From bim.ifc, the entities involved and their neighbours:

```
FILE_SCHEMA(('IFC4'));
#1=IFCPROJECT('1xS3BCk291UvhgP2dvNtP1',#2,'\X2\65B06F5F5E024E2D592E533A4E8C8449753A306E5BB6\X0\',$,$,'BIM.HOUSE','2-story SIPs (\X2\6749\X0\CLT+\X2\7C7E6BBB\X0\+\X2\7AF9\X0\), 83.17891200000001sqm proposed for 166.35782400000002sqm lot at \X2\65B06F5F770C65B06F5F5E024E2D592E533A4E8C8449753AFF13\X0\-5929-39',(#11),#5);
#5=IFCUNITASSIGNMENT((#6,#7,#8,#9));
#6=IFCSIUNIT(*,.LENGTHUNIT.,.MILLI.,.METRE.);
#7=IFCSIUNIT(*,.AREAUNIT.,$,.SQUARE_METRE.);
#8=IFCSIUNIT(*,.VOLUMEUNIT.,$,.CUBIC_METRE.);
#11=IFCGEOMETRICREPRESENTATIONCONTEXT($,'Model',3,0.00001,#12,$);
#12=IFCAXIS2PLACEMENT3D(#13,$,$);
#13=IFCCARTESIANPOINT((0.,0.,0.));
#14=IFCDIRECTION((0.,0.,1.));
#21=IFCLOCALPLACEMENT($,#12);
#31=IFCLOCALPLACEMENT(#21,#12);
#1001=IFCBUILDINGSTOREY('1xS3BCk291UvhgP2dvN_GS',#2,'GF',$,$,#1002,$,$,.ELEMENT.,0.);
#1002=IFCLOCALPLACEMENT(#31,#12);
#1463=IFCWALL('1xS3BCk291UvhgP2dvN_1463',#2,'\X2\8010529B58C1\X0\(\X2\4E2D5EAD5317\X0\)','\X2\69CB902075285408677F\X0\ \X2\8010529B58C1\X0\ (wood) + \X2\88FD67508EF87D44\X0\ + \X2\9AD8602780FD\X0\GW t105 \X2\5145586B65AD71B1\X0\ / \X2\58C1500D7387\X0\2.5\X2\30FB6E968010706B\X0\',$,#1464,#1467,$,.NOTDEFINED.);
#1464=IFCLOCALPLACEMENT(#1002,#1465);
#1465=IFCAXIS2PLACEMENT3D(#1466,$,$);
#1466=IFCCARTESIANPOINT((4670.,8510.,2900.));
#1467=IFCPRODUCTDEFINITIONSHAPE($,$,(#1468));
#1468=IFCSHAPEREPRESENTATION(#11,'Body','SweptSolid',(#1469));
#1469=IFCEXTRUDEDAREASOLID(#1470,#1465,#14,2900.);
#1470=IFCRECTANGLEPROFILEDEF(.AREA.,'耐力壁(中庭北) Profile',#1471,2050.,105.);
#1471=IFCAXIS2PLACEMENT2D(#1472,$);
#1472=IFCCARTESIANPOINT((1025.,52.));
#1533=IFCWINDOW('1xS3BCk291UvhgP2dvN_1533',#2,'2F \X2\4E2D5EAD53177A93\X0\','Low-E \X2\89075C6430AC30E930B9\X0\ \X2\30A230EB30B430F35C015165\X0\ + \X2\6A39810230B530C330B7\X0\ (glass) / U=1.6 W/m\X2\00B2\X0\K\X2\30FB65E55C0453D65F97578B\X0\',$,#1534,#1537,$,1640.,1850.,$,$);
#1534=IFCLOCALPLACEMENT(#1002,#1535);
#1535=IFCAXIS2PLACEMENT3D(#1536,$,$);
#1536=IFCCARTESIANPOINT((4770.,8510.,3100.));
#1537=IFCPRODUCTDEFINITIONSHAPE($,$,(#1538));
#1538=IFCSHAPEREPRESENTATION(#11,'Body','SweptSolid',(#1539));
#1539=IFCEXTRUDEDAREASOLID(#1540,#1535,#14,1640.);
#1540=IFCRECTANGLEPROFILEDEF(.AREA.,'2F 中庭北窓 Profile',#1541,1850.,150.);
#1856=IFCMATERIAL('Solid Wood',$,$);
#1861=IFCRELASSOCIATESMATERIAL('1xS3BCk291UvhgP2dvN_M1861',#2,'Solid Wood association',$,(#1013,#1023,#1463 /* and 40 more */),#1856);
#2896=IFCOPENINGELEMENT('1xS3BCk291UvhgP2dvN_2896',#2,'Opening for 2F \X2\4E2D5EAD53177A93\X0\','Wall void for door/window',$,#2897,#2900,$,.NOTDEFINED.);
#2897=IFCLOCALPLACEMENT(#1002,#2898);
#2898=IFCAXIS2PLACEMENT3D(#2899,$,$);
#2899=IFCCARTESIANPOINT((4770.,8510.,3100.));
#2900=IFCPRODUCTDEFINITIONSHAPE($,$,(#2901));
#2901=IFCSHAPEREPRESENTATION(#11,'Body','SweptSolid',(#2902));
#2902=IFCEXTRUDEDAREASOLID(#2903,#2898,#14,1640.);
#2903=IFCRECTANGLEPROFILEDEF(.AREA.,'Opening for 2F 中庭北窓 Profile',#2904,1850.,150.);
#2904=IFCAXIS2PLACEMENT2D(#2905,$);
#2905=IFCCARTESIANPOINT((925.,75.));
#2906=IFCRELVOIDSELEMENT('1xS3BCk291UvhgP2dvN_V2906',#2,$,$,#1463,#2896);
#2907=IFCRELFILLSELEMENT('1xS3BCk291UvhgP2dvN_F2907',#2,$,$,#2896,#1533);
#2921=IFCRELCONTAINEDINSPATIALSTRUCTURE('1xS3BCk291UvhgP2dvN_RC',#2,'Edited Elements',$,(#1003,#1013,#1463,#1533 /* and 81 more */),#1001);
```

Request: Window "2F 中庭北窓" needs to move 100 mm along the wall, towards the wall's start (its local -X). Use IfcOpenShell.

```python
import ifcopenshell
import ifcopenshell.api.geometry
import ifcopenshell.util.placement

model = ifcopenshell.open("bim.ifc")

window = model.by_guid("1xS3BCk291UvhgP2dvN_1533")
opening = window.FillsVoids[0].RelatingOpeningElement
wall = opening.VoidsElements[0].RelatingBuildingElement

wall_matrix = ifcopenshell.util.placement.get_local_placement(wall.ObjectPlacement)
shift = wall_matrix[:3, 0] * -100.0
before = ifcopenshell.util.placement.get_local_placement(window.ObjectPlacement)[:3, 3].copy()

# The window is not placed relative to its opening, so move both.
for product in (opening, window):
    matrix = ifcopenshell.util.placement.get_local_placement(product.ObjectPlacement)
    matrix[:3, 3] += shift
    ifcopenshell.api.geometry.edit_object_placement(model, product=product, matrix=matrix, is_si=False)

after = ifcopenshell.util.placement.get_local_placement(window.ObjectPlacement)[:3, 3]
print("window moved by", (after - before).round(3) + 0.0)

model.write("bim_edited.ifc")
```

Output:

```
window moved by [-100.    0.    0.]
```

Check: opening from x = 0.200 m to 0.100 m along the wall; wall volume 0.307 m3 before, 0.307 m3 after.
